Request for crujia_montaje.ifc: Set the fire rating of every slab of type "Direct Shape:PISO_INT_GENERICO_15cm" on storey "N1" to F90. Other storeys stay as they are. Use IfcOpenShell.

First a look at what the model holds.

```python
import ifcopenshell
import ifcopenshell.util.element

model = ifcopenshell.open("crujia_montaje.ifc")
print(model.schema)
storey = next(s for s in model.by_type("IfcBuildingStorey") if s.Name == "N1")
slabs = [e for e in ifcopenshell.util.element.get_decomposition(storey) if e.is_a("IfcSlab")]
seen = {}
for e in slabs:
    element_type = ifcopenshell.util.element.get_type(e)
    key = (element_type.Name if element_type != e and element_type else None, ifcopenshell.util.element.get_pset(e, "Pset_SlabCommon", "FireRating"))
    seen[key] = seen.get(key, 0) + 1
for (name, value), count in sorted(seen.items(), key=str):
    print(count, "x", name, "|", value)
```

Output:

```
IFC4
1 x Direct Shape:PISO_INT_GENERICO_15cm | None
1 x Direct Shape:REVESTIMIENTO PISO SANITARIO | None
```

```python
import ifcopenshell
import ifcopenshell.api.pset
import ifcopenshell.util.element

model = ifcopenshell.open("crujia_montaje.ifc")

storey = next(s for s in model.by_type("IfcBuildingStorey") if s.Name == "N1")
slabs = [e for e in ifcopenshell.util.element.get_decomposition(storey) if e.is_a("IfcSlab")]

count = 0
for e in slabs:
    element_type = ifcopenshell.util.element.get_type(e)
    if element_type in (None, e) or element_type.Name != "Direct Shape:PISO_INT_GENERICO_15cm":
        continue
    # add_pset returns the element's existing set when there is one.
    pset = ifcopenshell.api.pset.add_pset(model, product=e, name="Pset_SlabCommon")
    ifcopenshell.api.pset.edit_pset(model, pset=pset, properties={"FireRating": "F90"})
    count += 1

print(count, "slabs updated")

model.write("crujia_montaje_rev.ifc")
```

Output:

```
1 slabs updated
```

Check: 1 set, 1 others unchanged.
